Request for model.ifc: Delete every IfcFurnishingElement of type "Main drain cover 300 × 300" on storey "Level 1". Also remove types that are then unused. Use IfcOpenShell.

First a look at what the model holds.

```python
import ifcopenshell
import ifcopenshell.util.element

model = ifcopenshell.open("model.ifc")
print(model.schema)
storey = next(s for s in model.by_type("IfcBuildingStorey") if s.Name == "Level 1")
furniture = [e for e in ifcopenshell.util.element.get_decomposition(storey) if e.is_a("IfcFurnishingElement")]
seen = {}
for e in furniture:
    element_type = ifcopenshell.util.element.get_type(e)
    name = element_type.Name if element_type not in (None, e) else None
    seen[name] = seen.get(name, 0) + 1
for name, count in sorted(seen.items(), key=str):
    print(count, "x", name)
```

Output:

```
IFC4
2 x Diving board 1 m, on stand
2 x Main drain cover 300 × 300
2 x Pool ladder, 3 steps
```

```python
import ifcopenshell
import ifcopenshell.api.root
import ifcopenshell.util.element

model = ifcopenshell.open("model.ifc")

storey = next(s for s in model.by_type("IfcBuildingStorey") if s.Name == "Level 1")
furniture = [e for e in ifcopenshell.util.element.get_decomposition(storey) if e.is_a("IfcFurnishingElement")]
targets = [e for e in furniture if (t := ifcopenshell.util.element.get_type(e)) not in (None, e) and t.Name == "Main drain cover 300 × 300"]
types = {ifcopenshell.util.element.get_type(e) for e in targets} - {None, *targets}

for e in targets:
    ifcopenshell.api.root.remove_product(model, product=e)
print(len(targets), "removed")

unused = [t for t in types if not ifcopenshell.util.element.get_types(t)]
for t in unused:
    ifcopenshell.api.root.remove_product(model, product=t)
print(len(unused), "unused types removed")

model.write("model_updated.ifc")
```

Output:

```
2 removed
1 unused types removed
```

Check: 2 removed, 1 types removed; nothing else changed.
